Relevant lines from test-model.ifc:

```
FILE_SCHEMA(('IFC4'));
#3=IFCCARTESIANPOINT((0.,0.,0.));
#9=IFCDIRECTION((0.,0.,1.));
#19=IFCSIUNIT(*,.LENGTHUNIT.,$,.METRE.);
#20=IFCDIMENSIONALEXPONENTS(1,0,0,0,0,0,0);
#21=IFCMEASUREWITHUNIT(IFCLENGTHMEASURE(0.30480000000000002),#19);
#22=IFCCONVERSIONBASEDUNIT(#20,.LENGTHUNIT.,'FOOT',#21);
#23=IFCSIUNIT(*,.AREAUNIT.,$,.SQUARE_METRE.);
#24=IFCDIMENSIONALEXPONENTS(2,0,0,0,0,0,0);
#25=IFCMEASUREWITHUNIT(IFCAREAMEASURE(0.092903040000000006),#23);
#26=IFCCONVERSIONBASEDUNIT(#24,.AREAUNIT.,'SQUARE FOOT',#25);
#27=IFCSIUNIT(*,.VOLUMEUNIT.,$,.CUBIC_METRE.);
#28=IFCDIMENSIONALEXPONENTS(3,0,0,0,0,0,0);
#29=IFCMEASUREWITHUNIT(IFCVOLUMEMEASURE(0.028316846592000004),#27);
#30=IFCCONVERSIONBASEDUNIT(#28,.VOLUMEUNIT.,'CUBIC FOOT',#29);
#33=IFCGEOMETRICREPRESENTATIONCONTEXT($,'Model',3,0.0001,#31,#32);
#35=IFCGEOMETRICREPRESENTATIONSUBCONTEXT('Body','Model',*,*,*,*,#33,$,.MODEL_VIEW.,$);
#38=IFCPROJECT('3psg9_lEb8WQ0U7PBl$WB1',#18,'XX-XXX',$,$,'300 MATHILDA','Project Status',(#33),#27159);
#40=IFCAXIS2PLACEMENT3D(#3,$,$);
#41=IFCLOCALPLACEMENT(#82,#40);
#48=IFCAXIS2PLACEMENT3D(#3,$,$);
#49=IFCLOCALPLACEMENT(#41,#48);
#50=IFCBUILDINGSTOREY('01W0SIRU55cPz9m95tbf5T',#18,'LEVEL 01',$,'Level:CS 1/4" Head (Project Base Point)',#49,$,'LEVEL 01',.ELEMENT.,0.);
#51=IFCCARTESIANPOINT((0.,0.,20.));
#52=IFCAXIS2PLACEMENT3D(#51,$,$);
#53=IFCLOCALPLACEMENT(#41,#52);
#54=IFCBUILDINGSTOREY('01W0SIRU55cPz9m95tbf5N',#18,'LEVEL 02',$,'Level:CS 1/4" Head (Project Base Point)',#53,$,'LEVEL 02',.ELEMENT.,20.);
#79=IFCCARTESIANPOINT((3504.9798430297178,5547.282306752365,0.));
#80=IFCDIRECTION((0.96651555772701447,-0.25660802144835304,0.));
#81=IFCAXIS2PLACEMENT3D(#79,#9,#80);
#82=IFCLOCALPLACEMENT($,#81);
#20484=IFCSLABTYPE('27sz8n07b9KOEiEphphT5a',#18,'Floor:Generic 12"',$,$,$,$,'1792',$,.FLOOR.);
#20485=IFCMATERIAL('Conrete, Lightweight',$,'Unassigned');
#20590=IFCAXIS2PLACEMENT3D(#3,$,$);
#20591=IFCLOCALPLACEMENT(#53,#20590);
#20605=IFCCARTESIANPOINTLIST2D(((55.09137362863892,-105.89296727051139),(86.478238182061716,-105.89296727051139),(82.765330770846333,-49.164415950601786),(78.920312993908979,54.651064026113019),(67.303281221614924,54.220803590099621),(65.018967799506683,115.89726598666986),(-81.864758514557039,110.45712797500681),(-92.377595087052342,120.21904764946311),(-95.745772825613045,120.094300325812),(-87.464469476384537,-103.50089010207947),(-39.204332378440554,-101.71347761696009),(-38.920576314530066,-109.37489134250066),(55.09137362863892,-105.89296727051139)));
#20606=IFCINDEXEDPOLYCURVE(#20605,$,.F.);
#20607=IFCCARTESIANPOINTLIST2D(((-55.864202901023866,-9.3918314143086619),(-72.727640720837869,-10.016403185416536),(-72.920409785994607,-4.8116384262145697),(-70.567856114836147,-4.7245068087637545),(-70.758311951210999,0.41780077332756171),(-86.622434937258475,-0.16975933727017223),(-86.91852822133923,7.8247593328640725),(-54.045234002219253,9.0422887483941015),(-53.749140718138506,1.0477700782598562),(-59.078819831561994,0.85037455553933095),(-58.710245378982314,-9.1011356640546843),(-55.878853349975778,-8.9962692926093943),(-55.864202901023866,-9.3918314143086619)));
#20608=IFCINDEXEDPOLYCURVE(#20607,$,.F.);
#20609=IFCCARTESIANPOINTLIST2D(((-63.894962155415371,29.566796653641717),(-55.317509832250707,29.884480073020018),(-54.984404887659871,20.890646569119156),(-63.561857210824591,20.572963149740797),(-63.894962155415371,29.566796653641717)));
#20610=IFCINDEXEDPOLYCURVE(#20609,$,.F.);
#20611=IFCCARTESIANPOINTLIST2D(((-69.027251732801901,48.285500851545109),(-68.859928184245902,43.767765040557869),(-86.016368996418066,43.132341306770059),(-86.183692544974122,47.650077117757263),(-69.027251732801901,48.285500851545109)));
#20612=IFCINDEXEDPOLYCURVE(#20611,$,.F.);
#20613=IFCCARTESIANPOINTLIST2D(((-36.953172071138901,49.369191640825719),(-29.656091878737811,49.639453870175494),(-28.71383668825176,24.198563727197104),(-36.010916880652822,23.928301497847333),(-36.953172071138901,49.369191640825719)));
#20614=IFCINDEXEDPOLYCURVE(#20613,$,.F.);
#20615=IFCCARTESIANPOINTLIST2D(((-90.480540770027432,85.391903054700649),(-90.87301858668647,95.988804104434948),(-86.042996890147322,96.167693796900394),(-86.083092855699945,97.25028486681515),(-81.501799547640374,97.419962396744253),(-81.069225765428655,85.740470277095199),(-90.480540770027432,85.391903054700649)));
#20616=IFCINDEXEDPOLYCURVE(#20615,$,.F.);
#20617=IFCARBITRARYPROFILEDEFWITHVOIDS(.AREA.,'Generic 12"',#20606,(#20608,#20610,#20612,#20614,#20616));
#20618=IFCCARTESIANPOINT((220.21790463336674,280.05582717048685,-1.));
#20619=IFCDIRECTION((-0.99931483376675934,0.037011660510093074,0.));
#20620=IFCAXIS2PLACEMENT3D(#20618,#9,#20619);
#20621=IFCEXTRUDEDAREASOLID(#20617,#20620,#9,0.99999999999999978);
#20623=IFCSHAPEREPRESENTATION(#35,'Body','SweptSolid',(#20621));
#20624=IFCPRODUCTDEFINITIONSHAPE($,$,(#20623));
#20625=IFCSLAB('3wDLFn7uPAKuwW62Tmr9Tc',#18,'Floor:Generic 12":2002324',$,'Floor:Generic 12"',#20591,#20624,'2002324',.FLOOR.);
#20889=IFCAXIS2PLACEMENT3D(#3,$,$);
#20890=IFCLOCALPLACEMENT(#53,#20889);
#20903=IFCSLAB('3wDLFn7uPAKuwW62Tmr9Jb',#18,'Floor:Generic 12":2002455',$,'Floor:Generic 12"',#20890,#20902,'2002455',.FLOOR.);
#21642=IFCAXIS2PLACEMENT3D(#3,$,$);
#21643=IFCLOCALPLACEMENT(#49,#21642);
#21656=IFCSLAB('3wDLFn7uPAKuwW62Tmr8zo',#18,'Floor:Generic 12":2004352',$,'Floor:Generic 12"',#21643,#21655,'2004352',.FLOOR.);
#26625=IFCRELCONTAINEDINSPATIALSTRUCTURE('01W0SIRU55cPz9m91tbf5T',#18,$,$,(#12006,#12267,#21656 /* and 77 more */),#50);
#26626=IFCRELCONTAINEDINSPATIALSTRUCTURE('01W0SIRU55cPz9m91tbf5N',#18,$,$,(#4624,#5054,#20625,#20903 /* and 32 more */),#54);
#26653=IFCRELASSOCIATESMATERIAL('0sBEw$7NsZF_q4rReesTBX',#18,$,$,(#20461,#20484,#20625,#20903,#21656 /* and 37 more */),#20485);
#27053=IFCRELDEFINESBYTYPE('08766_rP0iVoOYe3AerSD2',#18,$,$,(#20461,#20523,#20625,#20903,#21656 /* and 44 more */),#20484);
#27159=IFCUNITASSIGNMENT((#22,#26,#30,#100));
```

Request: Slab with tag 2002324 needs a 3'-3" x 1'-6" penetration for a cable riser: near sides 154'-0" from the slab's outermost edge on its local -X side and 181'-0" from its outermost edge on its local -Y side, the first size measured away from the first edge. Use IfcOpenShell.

```python
import numpy as np
import ifcopenshell
import ifcopenshell.api.feature
import ifcopenshell.api.geometry
import ifcopenshell.api.root
import ifcopenshell.geom
import ifcopenshell.util.placement
import ifcopenshell.util.representation
import ifcopenshell.util.shape
import ifcopenshell.util.unit

model = ifcopenshell.open("test-model.ifc")
unit_scale = ifcopenshell.util.unit.calculate_unit_scale(model)
settings = ifcopenshell.geom.settings()


def volume(element):
    """Net volume in cubic metres, openings subtracted."""
    shape = ifcopenshell.geom.create_shape(settings, element)
    return ifcopenshell.util.shape.get_volume(shape.geometry)


slab = model.by_guid("3wDLFn7uPAKuwW62Tmr9Tc")
before = volume(slab)

# Extent in the slab's own axes, in metres. The edges named are its -X and -Y sides.
slab_shape = ifcopenshell.geom.create_shape(settings, slab)
vertices = ifcopenshell.util.shape.get_vertices(slab_shape.geometry)
x_min, y_min, bottom = vertices.min(axis=0)
top = vertices[:, 2].max()

opening = ifcopenshell.api.root.create_entity(model, ifc_class="IfcOpeningElement", name="Cable riser opening", predefined_type="OPENING")
context = ifcopenshell.util.representation.get_context(model, "Model", "Body", "MODEL_VIEW")
width, depth = 0.9906, 0.4572
outline = [(0.0, 0.0), (width, 0.0), (width, depth), (0.0, depth), (0.0, 0.0)]
# Overshoot both faces by 50 mm so the cut is clean.
shape = ifcopenshell.api.geometry.add_slab_representation(
    model, context=context, depth=top - bottom + 0.1, polyline=outline
)
ifcopenshell.api.geometry.assign_representation(model, product=opening, representation=shape)

matrix = ifcopenshell.util.placement.get_local_placement(slab.ObjectPlacement)
matrix[:, 3] = matrix @ np.append(np.array([x_min + 46.9392, y_min + 55.1688, bottom - 0.05]) / unit_scale, 1.0)
ifcopenshell.api.geometry.edit_object_placement(model, product=opening, matrix=matrix, is_si=False)
ifcopenshell.api.feature.add_feature(model, feature=opening, element=slab)

after = volume(slab)

print(f"slab volume {before:.3f} -> {after:.3f} m3")

model.write("test-model_v2.ifc")
```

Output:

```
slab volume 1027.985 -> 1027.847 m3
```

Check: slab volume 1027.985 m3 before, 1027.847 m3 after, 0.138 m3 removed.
